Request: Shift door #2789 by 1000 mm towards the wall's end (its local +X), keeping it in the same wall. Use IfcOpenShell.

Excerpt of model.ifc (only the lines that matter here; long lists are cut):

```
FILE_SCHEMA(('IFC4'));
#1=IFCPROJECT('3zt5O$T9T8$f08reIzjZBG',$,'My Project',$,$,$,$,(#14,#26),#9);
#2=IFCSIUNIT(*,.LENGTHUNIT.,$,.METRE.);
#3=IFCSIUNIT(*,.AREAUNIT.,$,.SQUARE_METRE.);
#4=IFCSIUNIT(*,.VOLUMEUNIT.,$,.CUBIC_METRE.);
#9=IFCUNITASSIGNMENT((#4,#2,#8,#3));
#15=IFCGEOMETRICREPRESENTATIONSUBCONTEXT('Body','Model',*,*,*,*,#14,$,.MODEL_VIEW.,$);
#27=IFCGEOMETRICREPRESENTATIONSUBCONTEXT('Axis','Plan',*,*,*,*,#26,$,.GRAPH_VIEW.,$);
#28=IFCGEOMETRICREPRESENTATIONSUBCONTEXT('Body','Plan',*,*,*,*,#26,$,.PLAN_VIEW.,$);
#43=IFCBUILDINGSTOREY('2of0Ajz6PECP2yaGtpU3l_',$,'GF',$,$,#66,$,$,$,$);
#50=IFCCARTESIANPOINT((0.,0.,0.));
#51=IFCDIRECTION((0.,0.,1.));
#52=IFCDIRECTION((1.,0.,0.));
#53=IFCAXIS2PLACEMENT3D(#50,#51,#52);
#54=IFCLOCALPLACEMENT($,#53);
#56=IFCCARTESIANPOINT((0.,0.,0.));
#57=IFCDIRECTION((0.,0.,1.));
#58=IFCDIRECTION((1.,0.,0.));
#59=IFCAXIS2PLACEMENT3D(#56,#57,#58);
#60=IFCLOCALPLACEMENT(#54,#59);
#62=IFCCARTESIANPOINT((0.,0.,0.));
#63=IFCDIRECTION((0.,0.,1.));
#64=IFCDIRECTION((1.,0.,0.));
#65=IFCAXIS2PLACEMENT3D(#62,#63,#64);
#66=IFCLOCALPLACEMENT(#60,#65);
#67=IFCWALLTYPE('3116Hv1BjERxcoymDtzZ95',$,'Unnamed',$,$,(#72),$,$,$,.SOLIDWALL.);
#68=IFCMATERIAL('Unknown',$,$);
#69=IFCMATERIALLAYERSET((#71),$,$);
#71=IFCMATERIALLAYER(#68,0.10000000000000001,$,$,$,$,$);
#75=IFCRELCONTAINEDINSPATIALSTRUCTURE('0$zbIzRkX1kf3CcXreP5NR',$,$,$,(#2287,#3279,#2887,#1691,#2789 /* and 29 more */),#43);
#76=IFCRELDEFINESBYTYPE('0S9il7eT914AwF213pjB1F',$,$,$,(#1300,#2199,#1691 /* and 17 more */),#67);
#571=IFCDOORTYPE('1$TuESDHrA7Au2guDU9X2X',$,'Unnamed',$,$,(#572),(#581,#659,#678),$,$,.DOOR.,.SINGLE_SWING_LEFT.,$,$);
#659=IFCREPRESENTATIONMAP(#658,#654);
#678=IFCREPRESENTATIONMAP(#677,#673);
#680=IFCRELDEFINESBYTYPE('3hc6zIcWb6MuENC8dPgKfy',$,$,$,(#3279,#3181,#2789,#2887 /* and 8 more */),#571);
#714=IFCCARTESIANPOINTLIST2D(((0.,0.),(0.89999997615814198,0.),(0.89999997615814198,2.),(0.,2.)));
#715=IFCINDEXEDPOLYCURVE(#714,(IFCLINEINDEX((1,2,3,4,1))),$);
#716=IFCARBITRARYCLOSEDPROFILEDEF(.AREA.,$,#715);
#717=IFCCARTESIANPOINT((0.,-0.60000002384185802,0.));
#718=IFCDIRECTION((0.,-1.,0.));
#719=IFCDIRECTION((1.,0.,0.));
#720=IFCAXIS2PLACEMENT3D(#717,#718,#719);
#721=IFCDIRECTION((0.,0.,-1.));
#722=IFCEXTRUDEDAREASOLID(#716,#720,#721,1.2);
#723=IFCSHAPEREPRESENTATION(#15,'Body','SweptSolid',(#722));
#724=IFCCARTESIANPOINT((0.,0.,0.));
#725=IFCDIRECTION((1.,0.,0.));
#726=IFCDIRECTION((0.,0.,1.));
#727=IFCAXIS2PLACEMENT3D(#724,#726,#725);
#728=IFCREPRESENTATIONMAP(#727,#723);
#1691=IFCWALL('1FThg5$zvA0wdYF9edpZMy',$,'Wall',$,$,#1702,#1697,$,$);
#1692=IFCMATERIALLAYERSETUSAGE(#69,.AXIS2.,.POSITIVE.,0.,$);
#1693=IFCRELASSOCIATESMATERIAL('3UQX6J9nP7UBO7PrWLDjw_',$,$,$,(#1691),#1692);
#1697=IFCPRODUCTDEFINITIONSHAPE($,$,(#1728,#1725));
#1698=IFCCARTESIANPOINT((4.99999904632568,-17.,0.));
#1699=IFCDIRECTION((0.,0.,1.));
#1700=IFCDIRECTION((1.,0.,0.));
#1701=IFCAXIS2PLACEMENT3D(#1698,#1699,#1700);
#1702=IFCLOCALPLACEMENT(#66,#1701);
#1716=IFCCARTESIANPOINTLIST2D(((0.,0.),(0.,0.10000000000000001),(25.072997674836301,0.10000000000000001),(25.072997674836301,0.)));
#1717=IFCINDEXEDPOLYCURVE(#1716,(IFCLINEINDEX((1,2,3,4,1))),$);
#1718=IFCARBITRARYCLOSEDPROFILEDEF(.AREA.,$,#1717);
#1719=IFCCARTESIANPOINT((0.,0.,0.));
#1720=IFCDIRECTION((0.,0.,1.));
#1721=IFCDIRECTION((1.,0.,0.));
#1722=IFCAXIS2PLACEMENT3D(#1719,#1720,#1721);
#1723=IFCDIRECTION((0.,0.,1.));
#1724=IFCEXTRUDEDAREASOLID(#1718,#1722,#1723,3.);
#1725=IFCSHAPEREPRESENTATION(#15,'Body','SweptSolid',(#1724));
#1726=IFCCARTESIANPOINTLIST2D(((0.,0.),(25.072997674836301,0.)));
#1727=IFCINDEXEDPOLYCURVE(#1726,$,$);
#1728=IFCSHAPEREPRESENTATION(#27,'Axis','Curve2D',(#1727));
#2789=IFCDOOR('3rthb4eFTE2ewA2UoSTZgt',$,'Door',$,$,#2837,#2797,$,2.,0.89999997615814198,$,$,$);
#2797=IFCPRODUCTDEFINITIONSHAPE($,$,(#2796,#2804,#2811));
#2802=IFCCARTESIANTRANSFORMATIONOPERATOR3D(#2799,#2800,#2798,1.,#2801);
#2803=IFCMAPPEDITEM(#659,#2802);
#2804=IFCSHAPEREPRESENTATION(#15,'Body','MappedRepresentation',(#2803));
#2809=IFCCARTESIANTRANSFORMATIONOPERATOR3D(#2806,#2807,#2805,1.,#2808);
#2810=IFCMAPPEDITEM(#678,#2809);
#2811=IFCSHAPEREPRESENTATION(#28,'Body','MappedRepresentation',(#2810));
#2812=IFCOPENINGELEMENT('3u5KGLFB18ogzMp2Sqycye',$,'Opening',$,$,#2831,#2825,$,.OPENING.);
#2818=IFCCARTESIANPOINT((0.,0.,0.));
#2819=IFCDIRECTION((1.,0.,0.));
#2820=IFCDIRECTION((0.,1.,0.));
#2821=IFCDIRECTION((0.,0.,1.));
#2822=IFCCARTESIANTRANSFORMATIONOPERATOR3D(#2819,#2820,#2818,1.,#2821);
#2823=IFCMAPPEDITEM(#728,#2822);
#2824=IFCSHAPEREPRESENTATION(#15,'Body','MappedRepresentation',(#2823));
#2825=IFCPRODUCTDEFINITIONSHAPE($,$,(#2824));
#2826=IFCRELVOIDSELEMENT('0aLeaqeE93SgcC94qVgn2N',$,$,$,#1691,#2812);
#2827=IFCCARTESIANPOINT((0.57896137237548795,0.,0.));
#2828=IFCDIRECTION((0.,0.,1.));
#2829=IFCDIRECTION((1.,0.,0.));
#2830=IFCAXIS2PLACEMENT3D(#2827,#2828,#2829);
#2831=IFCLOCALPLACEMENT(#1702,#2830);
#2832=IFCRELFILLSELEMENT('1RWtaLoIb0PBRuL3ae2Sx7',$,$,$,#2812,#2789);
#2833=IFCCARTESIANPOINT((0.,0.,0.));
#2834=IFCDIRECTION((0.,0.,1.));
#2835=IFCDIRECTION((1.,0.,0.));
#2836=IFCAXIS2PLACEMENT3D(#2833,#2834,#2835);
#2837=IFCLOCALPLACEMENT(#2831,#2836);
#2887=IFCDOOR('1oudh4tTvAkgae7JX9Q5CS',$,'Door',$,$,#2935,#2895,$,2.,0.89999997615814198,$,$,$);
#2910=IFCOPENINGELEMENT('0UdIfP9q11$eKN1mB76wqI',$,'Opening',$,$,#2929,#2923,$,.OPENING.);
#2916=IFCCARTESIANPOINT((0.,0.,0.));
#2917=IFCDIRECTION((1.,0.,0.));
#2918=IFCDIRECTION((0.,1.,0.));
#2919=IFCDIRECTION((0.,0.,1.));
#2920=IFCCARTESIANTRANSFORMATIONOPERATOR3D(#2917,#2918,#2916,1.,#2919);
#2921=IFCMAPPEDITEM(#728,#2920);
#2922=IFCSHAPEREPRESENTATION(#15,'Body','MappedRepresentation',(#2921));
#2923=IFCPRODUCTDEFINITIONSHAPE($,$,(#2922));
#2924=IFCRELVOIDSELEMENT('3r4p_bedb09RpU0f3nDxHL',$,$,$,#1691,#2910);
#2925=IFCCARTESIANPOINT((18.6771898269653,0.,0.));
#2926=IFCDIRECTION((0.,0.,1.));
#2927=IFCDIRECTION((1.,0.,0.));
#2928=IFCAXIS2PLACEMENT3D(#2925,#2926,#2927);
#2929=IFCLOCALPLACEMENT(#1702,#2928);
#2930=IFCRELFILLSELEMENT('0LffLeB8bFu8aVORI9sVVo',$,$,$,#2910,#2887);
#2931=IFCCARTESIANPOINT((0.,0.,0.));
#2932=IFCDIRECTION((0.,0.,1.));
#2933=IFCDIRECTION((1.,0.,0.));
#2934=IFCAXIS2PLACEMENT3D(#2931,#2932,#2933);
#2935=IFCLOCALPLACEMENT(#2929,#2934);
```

```python
import ifcopenshell
import ifcopenshell.api.geometry
import ifcopenshell.util.placement
import ifcopenshell.util.unit

model = ifcopenshell.open("model.ifc")
unit_scale = ifcopenshell.util.unit.calculate_unit_scale(model)

door = model.by_id(2789)
opening = door.FillsVoids[0].RelatingOpeningElement
wall = opening.VoidsElements[0].RelatingBuildingElement

wall_matrix = ifcopenshell.util.placement.get_local_placement(wall.ObjectPlacement)
shift = wall_matrix[:3, 0] * 1 / unit_scale
before = ifcopenshell.util.placement.get_local_placement(door.ObjectPlacement)[:3, 3].copy()

# The door is placed relative to its opening, so it follows when the opening moves.
matrix = ifcopenshell.util.placement.get_local_placement(opening.ObjectPlacement)
matrix[:3, 3] += shift
ifcopenshell.api.geometry.edit_object_placement(
    model, product=opening, matrix=matrix, is_si=False, should_transform_children=True
)

after = ifcopenshell.util.placement.get_local_placement(door.ObjectPlacement)[:3, 3]
print("door moved by", (after - before).round(3) + 0.0)

model.write("model_v2.ifc")
```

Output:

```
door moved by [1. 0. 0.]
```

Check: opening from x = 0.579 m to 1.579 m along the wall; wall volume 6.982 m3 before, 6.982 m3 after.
